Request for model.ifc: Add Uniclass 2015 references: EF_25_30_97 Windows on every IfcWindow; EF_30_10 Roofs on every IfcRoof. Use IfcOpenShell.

First a look at what the model holds.

```python
import ifcopenshell

model = ifcopenshell.open("model.ifc")
print(model.schema)
print("classifications:", [c.Name for c in model.by_type("IfcClassification")])
for ifc_class in ("IfcDoor", "IfcRoof", "IfcStair", "IfcWall", "IfcWindow"):
    print(ifc_class, len(model.by_type(ifc_class)))
```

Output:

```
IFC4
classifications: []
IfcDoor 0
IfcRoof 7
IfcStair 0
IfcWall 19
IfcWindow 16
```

```python
import ifcopenshell
import ifcopenshell.api.classification

model = ifcopenshell.open("model.ifc")

system = ifcopenshell.api.classification.add_classification(model, classification="Uniclass 2015")

codes = {
    "IfcWindow": ("EF_25_30_97", "Windows"),
    "IfcRoof": ("EF_30_10", "Roofs"),
}
for ifc_class, (code, name) in codes.items():
    products = model.by_type(ifc_class)
    ifcopenshell.api.classification.add_reference(
        model, products=products, classification=system, identification=code, name=name
    )
    print(code, len(products))

model.write("model_rev.ifc")
```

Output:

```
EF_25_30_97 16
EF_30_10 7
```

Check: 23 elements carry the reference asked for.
